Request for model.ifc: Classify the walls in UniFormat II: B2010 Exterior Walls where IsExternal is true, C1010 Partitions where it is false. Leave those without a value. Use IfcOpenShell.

First a look at what the model holds.

```python
import ifcopenshell
import ifcopenshell.util.element

model = ifcopenshell.open("model.ifc")
print(model.schema)
print("classifications:", [c.Name for c in model.by_type("IfcClassification")])
values = [ifcopenshell.util.element.get_pset(e, "Pset_WallCommon", "IsExternal") for e in model.by_type("IfcWall")]
for value in (True, False, None):
    print("IsExternal", value, values.count(value))
```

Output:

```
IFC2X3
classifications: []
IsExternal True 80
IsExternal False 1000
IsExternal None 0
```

```python
import ifcopenshell
import ifcopenshell.api.classification
import ifcopenshell.util.element

model = ifcopenshell.open("model.ifc")

# IFC2X3 requires Source and Edition and has no link from the project to the system.
system = model.create_entity("IfcClassification", Source="ASTM", Edition="E1557", Name="UniFormat II")

walls = model.by_type("IfcWall")
external = {e: ifcopenshell.util.element.get_pset(e, "Pset_WallCommon", "IsExternal") for e in walls}
for flag, code, name in ((True, "B2010", "Exterior Walls"), (False, "C1010", "Partitions")):
    products = [e for e in walls if external[e] is flag]
    ifcopenshell.api.classification.add_reference(
        model, products=products, classification=system, identification=code, name=name
    )
    print(code, len(products))

model.write("model_v2.ifc")
```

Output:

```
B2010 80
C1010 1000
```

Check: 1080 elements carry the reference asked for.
